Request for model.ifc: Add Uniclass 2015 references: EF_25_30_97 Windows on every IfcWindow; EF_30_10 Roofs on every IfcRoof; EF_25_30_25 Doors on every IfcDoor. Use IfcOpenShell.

First a look at what the model holds.

```python
import ifcopenshell

model = ifcopenshell.open("model.ifc")
print(model.schema)
print("classifications:", [c.Name for c in model.by_type("IfcClassification")])
for ifc_class in ("IfcDoor", "IfcRoof", "IfcStair", "IfcWall", "IfcWindow"):
    print(ifc_class, len(model.by_type(ifc_class)))
```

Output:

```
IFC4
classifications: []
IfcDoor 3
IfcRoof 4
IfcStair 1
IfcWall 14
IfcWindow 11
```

```python
import ifcopenshell
import ifcopenshell.api.classification

model = ifcopenshell.open("model.ifc")

system = ifcopenshell.api.classification.add_classification(model, classification="Uniclass 2015")

codes = {
    "IfcWindow": ("EF_25_30_97", "Windows"),
    "IfcRoof": ("EF_30_10", "Roofs"),
    "IfcDoor": ("EF_25_30_25", "Doors"),
}
for ifc_class, (code, name) in codes.items():
    products = model.by_type(ifc_class)
    ifcopenshell.api.classification.add_reference(
        model, products=products, classification=system, identification=code, name=name
    )
    print(code, len(products))

model.write("model_updated.ifc")
```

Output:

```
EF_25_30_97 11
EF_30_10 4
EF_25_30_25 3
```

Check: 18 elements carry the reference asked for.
